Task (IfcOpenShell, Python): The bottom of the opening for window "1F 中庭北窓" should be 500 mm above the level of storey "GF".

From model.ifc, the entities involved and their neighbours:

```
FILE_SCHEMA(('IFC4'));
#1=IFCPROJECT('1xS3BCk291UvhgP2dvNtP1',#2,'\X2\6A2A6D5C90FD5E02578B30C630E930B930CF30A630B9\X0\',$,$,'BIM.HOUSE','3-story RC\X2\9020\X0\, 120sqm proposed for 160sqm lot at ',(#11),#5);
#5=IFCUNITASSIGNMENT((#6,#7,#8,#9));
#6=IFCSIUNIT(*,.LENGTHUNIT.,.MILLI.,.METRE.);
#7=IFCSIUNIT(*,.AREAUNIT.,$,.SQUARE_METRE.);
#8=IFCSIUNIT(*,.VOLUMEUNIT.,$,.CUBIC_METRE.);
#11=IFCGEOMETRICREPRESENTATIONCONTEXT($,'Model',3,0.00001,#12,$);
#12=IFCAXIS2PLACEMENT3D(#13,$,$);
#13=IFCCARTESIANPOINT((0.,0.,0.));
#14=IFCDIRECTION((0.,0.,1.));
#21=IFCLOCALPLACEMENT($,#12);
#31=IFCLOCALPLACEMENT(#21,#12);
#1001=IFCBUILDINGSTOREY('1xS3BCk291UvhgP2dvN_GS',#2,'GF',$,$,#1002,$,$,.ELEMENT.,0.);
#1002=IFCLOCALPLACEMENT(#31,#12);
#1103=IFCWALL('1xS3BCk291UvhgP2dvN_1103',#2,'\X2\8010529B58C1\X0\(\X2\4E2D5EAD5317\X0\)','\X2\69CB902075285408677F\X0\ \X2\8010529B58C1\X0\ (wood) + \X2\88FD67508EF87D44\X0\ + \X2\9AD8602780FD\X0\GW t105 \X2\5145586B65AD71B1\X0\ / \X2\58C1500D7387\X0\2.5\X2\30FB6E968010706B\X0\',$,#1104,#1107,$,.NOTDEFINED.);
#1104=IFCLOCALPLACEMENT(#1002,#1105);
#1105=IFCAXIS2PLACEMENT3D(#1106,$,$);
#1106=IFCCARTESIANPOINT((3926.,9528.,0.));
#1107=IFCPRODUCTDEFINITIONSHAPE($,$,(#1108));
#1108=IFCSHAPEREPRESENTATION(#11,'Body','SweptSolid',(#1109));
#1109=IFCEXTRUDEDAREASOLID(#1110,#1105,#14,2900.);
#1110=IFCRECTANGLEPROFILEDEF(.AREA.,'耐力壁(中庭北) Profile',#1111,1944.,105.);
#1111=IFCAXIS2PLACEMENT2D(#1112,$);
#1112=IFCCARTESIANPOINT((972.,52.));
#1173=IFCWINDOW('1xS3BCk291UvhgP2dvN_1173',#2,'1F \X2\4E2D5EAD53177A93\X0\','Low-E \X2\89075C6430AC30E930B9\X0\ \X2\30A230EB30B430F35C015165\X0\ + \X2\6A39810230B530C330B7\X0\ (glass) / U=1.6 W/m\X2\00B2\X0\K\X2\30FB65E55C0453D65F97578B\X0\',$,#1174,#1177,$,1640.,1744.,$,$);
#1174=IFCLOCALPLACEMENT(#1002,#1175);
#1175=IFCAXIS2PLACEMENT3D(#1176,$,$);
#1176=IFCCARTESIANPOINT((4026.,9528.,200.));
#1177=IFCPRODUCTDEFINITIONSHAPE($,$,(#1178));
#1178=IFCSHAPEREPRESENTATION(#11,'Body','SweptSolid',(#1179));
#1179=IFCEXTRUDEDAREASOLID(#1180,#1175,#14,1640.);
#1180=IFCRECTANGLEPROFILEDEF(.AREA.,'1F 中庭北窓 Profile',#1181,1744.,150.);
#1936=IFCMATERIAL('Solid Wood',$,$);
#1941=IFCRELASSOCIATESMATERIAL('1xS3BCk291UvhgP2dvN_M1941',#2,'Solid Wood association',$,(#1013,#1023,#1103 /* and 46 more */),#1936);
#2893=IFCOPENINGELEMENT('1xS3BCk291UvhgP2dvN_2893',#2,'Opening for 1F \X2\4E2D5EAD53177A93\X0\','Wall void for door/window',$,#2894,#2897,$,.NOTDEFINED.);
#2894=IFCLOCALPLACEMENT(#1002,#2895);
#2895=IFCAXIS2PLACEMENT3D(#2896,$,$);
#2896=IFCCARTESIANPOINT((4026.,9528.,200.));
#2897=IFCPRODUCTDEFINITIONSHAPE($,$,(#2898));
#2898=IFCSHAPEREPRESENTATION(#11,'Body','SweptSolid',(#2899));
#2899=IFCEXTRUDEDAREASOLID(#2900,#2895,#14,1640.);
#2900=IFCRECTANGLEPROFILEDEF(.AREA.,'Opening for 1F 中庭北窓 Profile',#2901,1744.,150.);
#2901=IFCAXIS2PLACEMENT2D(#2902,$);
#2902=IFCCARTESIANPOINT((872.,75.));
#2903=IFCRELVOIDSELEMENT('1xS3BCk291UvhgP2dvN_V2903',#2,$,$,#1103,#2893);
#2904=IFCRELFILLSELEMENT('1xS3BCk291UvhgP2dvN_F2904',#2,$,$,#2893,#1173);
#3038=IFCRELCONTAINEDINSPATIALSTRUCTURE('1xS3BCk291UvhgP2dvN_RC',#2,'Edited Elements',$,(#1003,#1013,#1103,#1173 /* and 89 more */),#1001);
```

```python
import numpy as np
import ifcopenshell
import ifcopenshell.api.geometry
import ifcopenshell.geom
import ifcopenshell.util.element
import ifcopenshell.util.placement
import ifcopenshell.util.shape
import ifcopenshell.util.unit

model = ifcopenshell.open("model.ifc")
unit_scale = ifcopenshell.util.unit.calculate_unit_scale(model)

window = model.by_guid("1xS3BCk291UvhgP2dvN_1173")
opening = window.FillsVoids[0].RelatingOpeningElement
storey = ifcopenshell.util.element.get_container(window, ifc_class="IfcBuildingStorey")
level = ifcopenshell.util.placement.get_local_placement(storey.ObjectPlacement)[2, 3]

# The opening's origin need not be at the sill, so measure its lowest point.
shape = ifcopenshell.geom.create_shape(ifcopenshell.geom.settings(), opening)
bottom = ifcopenshell.util.shape.get_shape_bottom_elevation(shape, shape.geometry) / unit_scale
dz = level + 0.5 / unit_scale - bottom

shift = np.array([0.0, 0.0, dz])
# The window is not placed relative to its opening, so move both.
for product in (opening, window):
    matrix = ifcopenshell.util.placement.get_local_placement(product.ObjectPlacement)
    matrix[:3, 3] += shift
    ifcopenshell.api.geometry.edit_object_placement(model, product=product, matrix=matrix, is_si=False)

print(f"moved by {dz * unit_scale:+.3f} m")

model.write("model_rev.ifc")
```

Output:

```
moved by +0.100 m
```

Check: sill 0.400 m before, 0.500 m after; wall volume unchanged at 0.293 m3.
